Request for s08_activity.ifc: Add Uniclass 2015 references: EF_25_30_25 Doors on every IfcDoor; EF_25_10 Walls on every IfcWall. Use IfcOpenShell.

First a look at what the model holds.

```python
import ifcopenshell

model = ifcopenshell.open("s08_activity.ifc")
print(model.schema)
print("classifications:", [c.Name for c in model.by_type("IfcClassification")])
for ifc_class in ("IfcDoor", "IfcRoof", "IfcStair", "IfcWall", "IfcWindow"):
    print(ifc_class, len(model.by_type(ifc_class)))
```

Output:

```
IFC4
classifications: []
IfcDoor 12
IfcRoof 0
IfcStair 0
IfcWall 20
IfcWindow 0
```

```python
import ifcopenshell
import ifcopenshell.api.classification

model = ifcopenshell.open("s08_activity.ifc")

system = ifcopenshell.api.classification.add_classification(model, classification="Uniclass 2015")

codes = {
    "IfcDoor": ("EF_25_30_25", "Doors"),
    "IfcWall": ("EF_25_10", "Walls"),
}
for ifc_class, (code, name) in codes.items():
    products = model.by_type(ifc_class)
    ifcopenshell.api.classification.add_reference(
        model, products=products, classification=system, identification=code, name=name
    )
    print(code, len(products))

model.write("s08_activity_v2.ifc")
```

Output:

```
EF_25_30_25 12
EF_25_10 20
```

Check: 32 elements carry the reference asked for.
